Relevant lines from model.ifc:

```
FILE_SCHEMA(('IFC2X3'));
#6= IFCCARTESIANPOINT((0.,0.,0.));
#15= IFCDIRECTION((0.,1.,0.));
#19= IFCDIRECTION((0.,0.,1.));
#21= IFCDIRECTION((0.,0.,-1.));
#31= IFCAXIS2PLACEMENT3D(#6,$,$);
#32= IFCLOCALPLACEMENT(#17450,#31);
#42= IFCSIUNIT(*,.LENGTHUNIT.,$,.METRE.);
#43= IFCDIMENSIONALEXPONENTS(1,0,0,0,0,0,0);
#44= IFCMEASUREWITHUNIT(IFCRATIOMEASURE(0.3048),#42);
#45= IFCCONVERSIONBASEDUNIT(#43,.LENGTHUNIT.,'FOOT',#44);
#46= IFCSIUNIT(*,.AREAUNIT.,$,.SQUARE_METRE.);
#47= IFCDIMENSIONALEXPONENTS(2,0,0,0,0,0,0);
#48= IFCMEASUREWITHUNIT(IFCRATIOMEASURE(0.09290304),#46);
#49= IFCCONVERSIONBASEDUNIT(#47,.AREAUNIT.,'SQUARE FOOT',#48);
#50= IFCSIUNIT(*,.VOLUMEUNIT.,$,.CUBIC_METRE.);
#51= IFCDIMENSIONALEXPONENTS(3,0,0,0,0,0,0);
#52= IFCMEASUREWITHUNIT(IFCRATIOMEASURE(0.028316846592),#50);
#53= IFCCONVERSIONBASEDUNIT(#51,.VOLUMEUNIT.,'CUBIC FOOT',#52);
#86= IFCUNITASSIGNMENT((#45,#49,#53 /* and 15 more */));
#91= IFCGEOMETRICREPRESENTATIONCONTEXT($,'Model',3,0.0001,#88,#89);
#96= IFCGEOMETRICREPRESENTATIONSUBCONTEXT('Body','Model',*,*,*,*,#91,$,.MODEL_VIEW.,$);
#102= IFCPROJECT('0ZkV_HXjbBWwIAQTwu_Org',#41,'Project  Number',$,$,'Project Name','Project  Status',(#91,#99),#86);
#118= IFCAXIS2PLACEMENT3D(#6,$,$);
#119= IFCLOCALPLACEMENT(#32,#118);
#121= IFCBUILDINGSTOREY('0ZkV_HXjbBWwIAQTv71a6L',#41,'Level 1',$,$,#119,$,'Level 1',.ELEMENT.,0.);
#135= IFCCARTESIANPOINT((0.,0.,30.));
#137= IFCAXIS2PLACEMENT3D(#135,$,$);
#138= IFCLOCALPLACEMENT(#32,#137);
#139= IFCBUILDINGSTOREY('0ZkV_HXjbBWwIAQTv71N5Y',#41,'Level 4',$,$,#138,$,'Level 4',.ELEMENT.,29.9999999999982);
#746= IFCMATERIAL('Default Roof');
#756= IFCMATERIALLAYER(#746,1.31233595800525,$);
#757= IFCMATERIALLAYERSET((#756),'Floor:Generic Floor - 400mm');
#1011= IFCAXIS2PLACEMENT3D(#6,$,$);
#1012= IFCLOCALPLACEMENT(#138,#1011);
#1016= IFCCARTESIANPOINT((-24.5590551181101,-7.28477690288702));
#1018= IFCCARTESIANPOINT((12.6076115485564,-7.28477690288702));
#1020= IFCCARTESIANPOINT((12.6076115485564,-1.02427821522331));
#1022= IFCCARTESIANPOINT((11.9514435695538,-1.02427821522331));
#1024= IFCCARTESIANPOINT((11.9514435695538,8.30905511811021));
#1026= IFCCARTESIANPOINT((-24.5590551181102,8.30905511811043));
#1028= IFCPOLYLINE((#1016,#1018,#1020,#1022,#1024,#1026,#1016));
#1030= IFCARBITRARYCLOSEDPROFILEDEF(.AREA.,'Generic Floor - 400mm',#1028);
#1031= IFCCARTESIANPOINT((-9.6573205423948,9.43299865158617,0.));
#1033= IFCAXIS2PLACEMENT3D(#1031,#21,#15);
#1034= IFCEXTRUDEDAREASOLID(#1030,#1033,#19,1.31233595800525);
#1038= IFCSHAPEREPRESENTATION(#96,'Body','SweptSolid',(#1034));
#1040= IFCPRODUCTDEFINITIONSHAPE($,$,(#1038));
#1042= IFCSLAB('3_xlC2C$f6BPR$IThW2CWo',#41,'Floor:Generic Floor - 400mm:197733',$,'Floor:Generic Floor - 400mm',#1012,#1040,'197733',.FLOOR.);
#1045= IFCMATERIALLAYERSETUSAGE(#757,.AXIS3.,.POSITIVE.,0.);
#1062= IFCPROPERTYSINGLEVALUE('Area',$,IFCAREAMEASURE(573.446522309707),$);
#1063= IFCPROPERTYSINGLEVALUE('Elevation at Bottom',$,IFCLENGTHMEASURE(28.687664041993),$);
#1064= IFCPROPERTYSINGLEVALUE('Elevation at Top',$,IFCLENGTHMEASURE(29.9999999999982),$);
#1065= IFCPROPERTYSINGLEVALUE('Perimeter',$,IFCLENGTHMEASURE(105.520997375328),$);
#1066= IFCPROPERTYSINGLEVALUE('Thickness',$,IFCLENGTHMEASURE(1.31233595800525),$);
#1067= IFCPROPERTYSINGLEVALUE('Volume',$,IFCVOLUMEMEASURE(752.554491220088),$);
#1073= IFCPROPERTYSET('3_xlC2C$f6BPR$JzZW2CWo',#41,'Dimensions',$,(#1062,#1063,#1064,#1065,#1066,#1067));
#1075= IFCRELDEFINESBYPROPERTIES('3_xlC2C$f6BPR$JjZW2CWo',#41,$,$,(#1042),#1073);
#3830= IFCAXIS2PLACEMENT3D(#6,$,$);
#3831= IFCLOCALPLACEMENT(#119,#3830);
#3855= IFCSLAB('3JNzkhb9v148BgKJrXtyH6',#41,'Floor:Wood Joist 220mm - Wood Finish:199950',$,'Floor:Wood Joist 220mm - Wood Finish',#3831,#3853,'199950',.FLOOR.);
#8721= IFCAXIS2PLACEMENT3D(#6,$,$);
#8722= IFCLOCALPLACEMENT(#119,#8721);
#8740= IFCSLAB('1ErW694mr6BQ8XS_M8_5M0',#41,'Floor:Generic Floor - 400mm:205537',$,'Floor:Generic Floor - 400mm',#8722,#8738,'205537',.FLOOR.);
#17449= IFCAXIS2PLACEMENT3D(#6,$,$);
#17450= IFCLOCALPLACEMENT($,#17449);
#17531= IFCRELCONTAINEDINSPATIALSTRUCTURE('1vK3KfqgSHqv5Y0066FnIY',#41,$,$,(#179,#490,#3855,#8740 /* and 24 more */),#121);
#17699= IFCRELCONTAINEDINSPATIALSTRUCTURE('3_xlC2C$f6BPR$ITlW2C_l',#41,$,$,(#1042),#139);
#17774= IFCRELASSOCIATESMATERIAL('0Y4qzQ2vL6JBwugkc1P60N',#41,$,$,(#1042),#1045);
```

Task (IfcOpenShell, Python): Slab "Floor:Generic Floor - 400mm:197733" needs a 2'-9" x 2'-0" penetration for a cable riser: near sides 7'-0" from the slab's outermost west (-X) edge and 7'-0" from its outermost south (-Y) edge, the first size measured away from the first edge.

```python
import numpy as np
import ifcopenshell
import ifcopenshell.api.feature
import ifcopenshell.api.geometry
import ifcopenshell.api.pset
import ifcopenshell.api.root
import ifcopenshell.geom
import ifcopenshell.util.element
import ifcopenshell.util.placement
import ifcopenshell.util.representation
import ifcopenshell.util.shape
import ifcopenshell.util.unit

model = ifcopenshell.open("model.ifc")
unit_scale = ifcopenshell.util.unit.calculate_unit_scale(model)
area_scale = ifcopenshell.util.unit.calculate_unit_scale(model, "AREAUNIT")
volume_scale = ifcopenshell.util.unit.calculate_unit_scale(model, "VOLUMEUNIT")
settings = ifcopenshell.geom.settings()


def volume(element):
    """Net volume in cubic metres, openings subtracted."""
    shape = ifcopenshell.geom.create_shape(settings, element)
    return ifcopenshell.util.shape.get_volume(shape.geometry)


slab = model.by_id(1042)
before = volume(slab)

# Extent in the slab's own axes, in metres. The edges named are its -X and -Y sides.
slab_shape = ifcopenshell.geom.create_shape(settings, slab)
vertices = ifcopenshell.util.shape.get_vertices(slab_shape.geometry)
x_min, y_min, bottom = vertices.min(axis=0)
top = vertices[:, 2].max()

opening = ifcopenshell.api.root.create_entity(model, ifc_class="IfcOpeningElement", name="Cable riser opening")
context = ifcopenshell.util.representation.get_context(model, "Model", "Body", "MODEL_VIEW")
width, depth = 0.8382, 0.6096
outline = [(0.0, 0.0), (width, 0.0), (width, depth), (0.0, depth), (0.0, 0.0)]
# Overshoot both faces by 50 mm so the cut is clean.
shape = ifcopenshell.api.geometry.add_slab_representation(
    model, context=context, depth=top - bottom + 0.1, polyline=outline
)
ifcopenshell.api.geometry.assign_representation(model, product=opening, representation=shape)

matrix = ifcopenshell.util.placement.get_local_placement(slab.ObjectPlacement)
matrix[:, 3] = matrix @ np.append(np.array([x_min + 2.1336, y_min + 2.1336, bottom - 0.05]) / unit_scale, 1.0)
ifcopenshell.api.geometry.edit_object_placement(model, product=opening, matrix=matrix, is_si=False)
ifcopenshell.api.feature.add_feature(model, feature=opening, element=slab)

after = volume(slab)

# Update the slab's stored quantities.
pset = model.by_id(ifcopenshell.util.element.get_pset(slab, "Dimensions", should_inherit=False)["id"])
ifcopenshell.api.pset.edit_pset(model, pset=pset, properties={
    "Area": model.create_entity("IfcAreaMeasure", after / (top - bottom) / area_scale),
    "Volume": model.create_entity("IfcVolumeMeasure", after / volume_scale),
})

print(f"slab volume {before:.3f} -> {after:.3f} m3")

model.write("model-out.ifc")
```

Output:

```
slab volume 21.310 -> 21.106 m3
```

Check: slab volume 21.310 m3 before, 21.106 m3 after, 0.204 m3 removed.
